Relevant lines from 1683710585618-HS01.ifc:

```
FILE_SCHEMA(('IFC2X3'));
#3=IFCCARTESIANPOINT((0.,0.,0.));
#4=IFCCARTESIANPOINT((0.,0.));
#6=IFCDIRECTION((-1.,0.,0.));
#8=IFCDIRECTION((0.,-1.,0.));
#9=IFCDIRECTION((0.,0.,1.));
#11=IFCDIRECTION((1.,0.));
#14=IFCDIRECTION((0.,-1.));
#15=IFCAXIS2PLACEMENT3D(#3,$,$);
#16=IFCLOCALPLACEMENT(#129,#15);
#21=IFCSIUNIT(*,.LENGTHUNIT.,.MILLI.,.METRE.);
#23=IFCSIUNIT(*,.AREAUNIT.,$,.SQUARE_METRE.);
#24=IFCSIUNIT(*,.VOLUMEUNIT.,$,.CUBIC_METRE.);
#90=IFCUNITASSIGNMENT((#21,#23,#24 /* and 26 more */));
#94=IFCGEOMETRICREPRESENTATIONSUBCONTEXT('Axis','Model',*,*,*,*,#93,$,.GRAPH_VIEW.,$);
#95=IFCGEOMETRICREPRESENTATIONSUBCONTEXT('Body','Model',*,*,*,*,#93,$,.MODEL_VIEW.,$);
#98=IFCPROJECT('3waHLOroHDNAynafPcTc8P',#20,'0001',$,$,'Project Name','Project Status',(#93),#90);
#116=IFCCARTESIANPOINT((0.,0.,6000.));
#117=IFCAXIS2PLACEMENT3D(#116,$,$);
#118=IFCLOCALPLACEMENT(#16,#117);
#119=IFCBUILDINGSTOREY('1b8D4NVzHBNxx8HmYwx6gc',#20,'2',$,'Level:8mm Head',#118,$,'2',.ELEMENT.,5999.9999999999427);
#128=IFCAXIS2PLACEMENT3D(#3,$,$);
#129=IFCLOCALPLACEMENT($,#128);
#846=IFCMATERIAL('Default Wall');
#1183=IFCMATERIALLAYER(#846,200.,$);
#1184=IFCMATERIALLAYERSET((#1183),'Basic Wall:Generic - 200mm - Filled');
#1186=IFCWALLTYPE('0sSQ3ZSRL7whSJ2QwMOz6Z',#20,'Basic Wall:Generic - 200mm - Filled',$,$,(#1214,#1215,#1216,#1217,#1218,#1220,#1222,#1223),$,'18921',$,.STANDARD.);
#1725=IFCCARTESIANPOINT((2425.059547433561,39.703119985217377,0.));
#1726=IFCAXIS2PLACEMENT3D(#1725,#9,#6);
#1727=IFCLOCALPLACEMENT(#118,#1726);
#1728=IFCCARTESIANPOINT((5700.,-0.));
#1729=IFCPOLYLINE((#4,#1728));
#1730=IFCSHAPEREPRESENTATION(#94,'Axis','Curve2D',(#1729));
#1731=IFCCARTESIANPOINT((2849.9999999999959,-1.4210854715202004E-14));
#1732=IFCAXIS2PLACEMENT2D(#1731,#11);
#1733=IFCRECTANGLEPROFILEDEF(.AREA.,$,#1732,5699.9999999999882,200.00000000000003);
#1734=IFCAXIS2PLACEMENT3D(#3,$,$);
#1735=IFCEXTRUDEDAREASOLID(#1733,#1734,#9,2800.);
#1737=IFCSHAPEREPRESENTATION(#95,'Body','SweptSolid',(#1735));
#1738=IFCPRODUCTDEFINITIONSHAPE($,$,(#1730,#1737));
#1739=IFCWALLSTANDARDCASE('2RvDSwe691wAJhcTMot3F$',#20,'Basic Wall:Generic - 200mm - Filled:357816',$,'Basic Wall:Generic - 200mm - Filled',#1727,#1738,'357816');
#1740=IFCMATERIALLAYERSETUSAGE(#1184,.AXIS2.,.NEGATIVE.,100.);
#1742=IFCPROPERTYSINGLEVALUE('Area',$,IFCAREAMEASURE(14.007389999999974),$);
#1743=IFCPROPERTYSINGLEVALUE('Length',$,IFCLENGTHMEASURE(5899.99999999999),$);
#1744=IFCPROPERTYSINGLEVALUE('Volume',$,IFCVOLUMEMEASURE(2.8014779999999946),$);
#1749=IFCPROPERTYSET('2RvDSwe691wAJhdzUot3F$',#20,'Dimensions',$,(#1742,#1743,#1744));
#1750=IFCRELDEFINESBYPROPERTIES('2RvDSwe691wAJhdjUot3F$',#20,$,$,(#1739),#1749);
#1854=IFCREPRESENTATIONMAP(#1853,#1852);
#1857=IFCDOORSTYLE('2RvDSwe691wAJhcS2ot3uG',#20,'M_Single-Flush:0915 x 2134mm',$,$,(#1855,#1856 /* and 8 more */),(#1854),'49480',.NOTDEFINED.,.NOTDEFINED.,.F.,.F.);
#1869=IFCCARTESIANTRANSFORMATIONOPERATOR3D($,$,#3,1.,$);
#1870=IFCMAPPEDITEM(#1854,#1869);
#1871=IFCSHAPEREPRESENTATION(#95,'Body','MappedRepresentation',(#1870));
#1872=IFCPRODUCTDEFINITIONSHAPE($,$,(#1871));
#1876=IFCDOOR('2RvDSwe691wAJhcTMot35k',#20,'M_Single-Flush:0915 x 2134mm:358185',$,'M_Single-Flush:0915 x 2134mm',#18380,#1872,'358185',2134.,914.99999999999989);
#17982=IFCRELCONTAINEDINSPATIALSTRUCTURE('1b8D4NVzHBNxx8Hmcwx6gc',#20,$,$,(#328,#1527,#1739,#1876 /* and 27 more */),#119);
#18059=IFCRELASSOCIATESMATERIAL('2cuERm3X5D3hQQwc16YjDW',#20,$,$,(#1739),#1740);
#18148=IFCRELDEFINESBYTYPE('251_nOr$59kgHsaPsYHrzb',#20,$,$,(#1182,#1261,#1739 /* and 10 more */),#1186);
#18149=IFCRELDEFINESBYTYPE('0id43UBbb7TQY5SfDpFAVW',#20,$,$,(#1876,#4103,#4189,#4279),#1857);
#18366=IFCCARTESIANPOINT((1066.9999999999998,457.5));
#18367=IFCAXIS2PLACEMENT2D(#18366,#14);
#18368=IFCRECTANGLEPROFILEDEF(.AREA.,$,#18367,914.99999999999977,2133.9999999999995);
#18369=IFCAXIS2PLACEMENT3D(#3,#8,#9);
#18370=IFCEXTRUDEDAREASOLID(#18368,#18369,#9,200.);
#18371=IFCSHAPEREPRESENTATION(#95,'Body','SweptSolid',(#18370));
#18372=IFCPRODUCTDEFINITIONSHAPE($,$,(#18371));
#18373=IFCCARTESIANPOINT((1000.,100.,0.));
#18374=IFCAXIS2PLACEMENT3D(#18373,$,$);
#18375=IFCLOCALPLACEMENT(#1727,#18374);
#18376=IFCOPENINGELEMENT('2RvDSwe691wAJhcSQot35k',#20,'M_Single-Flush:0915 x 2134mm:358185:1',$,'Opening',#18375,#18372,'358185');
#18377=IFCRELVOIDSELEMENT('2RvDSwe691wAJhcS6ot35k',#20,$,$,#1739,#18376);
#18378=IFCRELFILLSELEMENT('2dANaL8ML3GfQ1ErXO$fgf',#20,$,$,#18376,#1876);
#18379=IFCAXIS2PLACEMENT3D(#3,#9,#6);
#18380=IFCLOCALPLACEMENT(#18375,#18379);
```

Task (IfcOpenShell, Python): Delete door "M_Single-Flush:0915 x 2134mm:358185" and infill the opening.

```python
import ifcopenshell
import ifcopenshell.api.feature
import ifcopenshell.api.pset
import ifcopenshell.api.root
import ifcopenshell.geom
import ifcopenshell.util.element
import ifcopenshell.util.shape
import ifcopenshell.util.unit

model = ifcopenshell.open("1683710585618-HS01.ifc")
area_scale = ifcopenshell.util.unit.calculate_unit_scale(model, "AREAUNIT")
volume_scale = ifcopenshell.util.unit.calculate_unit_scale(model, "VOLUMEUNIT")
settings = ifcopenshell.geom.settings()


def volume(element):
    """Net volume in cubic metres, openings subtracted."""
    shape = ifcopenshell.geom.create_shape(settings, element)
    return ifcopenshell.util.shape.get_volume(shape.geometry)


door = model.by_guid("2RvDSwe691wAJhcTMot35k")
opening = door.FillsVoids[0].RelatingOpeningElement
wall = opening.VoidsElements[0].RelatingBuildingElement
before = volume(wall)

ifcopenshell.api.root.remove_product(model, product=door)
ifcopenshell.api.feature.remove_feature(model, feature=opening)

after = volume(wall)
thickness = 0.2  # wall thickness in metres

# Update the wall's stored quantities.
pset = model.by_id(ifcopenshell.util.element.get_pset(wall, "Dimensions", should_inherit=False)["id"])
ifcopenshell.api.pset.edit_pset(model, pset=pset, properties={
    "Area": model.create_entity("IfcAreaMeasure", after / thickness / area_scale),
    "Volume": model.create_entity("IfcVolumeMeasure", after / volume_scale),
})

print(f"wall volume {before:.3f} -> {after:.3f} m3")

model.write("1683710585618-HS01_edited.ifc")
```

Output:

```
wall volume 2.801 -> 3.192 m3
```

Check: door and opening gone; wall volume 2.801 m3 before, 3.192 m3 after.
